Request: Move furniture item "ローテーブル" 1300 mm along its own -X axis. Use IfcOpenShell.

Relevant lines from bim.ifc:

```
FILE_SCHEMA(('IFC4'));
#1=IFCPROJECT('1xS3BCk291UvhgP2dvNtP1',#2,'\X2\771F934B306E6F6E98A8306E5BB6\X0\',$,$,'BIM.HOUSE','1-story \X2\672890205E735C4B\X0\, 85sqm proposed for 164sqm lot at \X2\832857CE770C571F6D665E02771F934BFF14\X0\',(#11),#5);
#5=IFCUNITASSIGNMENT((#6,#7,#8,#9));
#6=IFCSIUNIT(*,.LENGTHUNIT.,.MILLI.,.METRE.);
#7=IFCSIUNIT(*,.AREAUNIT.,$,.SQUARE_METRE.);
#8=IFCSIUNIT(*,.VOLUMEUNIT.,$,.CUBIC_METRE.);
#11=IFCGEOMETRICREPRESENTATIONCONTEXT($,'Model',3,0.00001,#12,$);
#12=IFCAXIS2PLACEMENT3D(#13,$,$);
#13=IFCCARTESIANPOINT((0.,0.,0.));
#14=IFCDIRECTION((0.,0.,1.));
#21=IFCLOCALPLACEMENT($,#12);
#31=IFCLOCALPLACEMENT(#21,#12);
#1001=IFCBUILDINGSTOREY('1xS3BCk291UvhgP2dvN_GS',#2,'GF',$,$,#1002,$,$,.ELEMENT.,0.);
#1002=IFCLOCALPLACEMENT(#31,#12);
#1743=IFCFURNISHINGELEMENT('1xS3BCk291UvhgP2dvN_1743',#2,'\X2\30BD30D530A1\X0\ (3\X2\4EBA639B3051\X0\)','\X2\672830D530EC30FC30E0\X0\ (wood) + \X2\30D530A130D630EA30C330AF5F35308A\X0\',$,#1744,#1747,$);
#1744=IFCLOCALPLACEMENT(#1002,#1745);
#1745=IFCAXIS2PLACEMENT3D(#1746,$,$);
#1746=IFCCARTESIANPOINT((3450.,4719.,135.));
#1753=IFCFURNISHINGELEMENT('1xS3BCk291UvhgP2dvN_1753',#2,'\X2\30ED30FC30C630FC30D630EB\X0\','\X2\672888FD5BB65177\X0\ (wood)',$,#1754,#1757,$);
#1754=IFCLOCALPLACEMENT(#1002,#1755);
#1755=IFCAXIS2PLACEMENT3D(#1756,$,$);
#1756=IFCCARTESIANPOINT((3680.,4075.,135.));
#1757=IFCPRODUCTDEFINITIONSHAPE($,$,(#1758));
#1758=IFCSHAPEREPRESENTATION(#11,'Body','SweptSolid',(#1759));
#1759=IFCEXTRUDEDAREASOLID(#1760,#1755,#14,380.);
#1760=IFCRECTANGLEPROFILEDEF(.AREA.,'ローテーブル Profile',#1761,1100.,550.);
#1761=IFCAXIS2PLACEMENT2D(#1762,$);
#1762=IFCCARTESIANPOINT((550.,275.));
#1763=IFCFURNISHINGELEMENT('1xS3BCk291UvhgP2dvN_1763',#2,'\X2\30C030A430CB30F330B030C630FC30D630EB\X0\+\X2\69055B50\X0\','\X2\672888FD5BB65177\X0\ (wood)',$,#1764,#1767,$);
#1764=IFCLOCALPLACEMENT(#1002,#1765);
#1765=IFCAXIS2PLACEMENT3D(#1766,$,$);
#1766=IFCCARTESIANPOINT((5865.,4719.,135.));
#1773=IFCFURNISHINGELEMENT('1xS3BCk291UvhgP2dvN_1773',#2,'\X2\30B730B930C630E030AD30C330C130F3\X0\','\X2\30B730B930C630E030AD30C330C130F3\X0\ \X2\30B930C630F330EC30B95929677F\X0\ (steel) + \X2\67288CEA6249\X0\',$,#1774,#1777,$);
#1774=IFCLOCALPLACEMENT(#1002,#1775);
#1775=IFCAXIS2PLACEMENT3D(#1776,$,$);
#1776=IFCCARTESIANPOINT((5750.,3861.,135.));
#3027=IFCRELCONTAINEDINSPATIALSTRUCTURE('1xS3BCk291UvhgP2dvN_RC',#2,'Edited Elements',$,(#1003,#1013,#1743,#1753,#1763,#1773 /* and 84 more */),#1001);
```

```python
import ifcopenshell
import ifcopenshell.api.geometry
import ifcopenshell.util.placement
import ifcopenshell.util.unit

model = ifcopenshell.open("bim.ifc")
unit_scale = ifcopenshell.util.unit.calculate_unit_scale(model)

item = model.by_guid("1xS3BCk291UvhgP2dvN_1753")
matrix = ifcopenshell.util.placement.get_local_placement(item.ObjectPlacement)
matrix[:3, 3] -= matrix[:3, 0] * 1.3 / unit_scale
ifcopenshell.api.geometry.edit_object_placement(model, product=item, matrix=matrix, is_si=False)

print(ifcopenshell.util.placement.get_local_placement(item.ObjectPlacement).round(3) + 0.0)

model.write("bim_rev.ifc")
```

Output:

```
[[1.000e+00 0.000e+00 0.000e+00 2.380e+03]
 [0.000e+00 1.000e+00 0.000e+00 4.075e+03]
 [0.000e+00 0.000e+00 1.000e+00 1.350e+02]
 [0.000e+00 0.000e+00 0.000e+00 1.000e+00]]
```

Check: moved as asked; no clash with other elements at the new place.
